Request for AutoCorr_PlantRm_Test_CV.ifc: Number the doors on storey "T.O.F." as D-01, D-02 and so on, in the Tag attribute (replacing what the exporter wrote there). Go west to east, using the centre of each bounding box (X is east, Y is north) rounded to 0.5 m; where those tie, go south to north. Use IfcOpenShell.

First a look at what the model holds.

```python
import ifcopenshell
import ifcopenshell.util.element
import ifcopenshell.util.placement

model = ifcopenshell.open("AutoCorr_PlantRm_Test_CV.ifc")
print(model.schema)
storey = next(s for s in model.by_type("IfcBuildingStorey") if s.Name == "T.O.F.")
doors = [e for e in ifcopenshell.util.element.get_decomposition(storey) if e.is_a("IfcDoor")]
for e in sorted(doors, key=lambda e: e.id()):
    origin = ifcopenshell.util.placement.get_local_placement(e.ObjectPlacement)[:3, 3]
    print(e.id(), e.Tag, e.Name, origin.round(2) + 0.0, sep=" | ")
```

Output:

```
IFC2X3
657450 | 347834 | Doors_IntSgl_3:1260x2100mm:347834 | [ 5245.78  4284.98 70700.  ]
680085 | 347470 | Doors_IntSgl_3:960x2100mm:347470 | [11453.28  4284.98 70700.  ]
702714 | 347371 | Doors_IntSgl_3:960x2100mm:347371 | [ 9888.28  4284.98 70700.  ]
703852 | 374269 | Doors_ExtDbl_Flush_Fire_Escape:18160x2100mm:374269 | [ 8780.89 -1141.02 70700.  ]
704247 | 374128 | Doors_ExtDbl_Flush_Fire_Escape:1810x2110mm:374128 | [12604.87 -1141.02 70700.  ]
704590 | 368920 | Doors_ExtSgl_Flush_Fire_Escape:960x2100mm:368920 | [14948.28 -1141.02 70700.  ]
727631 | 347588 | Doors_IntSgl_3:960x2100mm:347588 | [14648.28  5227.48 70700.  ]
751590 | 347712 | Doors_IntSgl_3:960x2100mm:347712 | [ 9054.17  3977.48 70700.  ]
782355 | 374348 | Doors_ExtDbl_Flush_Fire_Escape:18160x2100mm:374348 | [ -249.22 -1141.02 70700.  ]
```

```python
import ifcopenshell
import ifcopenshell.geom
import ifcopenshell.util.element
import ifcopenshell.util.shape

model = ifcopenshell.open("AutoCorr_PlantRm_Test_CV.ifc")
settings = ifcopenshell.geom.settings()
settings.set("use-world-coords", True)


def centre(element):
    shape = ifcopenshell.geom.create_shape(settings, element)
    return ifcopenshell.util.shape.get_bbox_centroid(shape.geometry)


storey = next(s for s in model.by_type("IfcBuildingStorey") if s.Name == "T.O.F.")
doors = [e for e in ifcopenshell.util.element.get_decomposition(storey) if e.is_a("IfcDoor")]

# Insertion points can sit at a corner or the storey origin, so sort by the geometry (in metres).
centres = {e: centre(e) for e in doors}
doors.sort(key=lambda e: (round(centres[e][0] / 0.5), centres[e][1]))

for i, e in enumerate(doors, start=1):
    number = f"D-{i:02d}"
    e.Tag = number
    print(e.id(), number)

model.write("AutoCorr_PlantRm_Test_CV_updated.ifc")
```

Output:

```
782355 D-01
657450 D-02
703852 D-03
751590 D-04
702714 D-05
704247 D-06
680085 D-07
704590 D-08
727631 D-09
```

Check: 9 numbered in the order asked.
